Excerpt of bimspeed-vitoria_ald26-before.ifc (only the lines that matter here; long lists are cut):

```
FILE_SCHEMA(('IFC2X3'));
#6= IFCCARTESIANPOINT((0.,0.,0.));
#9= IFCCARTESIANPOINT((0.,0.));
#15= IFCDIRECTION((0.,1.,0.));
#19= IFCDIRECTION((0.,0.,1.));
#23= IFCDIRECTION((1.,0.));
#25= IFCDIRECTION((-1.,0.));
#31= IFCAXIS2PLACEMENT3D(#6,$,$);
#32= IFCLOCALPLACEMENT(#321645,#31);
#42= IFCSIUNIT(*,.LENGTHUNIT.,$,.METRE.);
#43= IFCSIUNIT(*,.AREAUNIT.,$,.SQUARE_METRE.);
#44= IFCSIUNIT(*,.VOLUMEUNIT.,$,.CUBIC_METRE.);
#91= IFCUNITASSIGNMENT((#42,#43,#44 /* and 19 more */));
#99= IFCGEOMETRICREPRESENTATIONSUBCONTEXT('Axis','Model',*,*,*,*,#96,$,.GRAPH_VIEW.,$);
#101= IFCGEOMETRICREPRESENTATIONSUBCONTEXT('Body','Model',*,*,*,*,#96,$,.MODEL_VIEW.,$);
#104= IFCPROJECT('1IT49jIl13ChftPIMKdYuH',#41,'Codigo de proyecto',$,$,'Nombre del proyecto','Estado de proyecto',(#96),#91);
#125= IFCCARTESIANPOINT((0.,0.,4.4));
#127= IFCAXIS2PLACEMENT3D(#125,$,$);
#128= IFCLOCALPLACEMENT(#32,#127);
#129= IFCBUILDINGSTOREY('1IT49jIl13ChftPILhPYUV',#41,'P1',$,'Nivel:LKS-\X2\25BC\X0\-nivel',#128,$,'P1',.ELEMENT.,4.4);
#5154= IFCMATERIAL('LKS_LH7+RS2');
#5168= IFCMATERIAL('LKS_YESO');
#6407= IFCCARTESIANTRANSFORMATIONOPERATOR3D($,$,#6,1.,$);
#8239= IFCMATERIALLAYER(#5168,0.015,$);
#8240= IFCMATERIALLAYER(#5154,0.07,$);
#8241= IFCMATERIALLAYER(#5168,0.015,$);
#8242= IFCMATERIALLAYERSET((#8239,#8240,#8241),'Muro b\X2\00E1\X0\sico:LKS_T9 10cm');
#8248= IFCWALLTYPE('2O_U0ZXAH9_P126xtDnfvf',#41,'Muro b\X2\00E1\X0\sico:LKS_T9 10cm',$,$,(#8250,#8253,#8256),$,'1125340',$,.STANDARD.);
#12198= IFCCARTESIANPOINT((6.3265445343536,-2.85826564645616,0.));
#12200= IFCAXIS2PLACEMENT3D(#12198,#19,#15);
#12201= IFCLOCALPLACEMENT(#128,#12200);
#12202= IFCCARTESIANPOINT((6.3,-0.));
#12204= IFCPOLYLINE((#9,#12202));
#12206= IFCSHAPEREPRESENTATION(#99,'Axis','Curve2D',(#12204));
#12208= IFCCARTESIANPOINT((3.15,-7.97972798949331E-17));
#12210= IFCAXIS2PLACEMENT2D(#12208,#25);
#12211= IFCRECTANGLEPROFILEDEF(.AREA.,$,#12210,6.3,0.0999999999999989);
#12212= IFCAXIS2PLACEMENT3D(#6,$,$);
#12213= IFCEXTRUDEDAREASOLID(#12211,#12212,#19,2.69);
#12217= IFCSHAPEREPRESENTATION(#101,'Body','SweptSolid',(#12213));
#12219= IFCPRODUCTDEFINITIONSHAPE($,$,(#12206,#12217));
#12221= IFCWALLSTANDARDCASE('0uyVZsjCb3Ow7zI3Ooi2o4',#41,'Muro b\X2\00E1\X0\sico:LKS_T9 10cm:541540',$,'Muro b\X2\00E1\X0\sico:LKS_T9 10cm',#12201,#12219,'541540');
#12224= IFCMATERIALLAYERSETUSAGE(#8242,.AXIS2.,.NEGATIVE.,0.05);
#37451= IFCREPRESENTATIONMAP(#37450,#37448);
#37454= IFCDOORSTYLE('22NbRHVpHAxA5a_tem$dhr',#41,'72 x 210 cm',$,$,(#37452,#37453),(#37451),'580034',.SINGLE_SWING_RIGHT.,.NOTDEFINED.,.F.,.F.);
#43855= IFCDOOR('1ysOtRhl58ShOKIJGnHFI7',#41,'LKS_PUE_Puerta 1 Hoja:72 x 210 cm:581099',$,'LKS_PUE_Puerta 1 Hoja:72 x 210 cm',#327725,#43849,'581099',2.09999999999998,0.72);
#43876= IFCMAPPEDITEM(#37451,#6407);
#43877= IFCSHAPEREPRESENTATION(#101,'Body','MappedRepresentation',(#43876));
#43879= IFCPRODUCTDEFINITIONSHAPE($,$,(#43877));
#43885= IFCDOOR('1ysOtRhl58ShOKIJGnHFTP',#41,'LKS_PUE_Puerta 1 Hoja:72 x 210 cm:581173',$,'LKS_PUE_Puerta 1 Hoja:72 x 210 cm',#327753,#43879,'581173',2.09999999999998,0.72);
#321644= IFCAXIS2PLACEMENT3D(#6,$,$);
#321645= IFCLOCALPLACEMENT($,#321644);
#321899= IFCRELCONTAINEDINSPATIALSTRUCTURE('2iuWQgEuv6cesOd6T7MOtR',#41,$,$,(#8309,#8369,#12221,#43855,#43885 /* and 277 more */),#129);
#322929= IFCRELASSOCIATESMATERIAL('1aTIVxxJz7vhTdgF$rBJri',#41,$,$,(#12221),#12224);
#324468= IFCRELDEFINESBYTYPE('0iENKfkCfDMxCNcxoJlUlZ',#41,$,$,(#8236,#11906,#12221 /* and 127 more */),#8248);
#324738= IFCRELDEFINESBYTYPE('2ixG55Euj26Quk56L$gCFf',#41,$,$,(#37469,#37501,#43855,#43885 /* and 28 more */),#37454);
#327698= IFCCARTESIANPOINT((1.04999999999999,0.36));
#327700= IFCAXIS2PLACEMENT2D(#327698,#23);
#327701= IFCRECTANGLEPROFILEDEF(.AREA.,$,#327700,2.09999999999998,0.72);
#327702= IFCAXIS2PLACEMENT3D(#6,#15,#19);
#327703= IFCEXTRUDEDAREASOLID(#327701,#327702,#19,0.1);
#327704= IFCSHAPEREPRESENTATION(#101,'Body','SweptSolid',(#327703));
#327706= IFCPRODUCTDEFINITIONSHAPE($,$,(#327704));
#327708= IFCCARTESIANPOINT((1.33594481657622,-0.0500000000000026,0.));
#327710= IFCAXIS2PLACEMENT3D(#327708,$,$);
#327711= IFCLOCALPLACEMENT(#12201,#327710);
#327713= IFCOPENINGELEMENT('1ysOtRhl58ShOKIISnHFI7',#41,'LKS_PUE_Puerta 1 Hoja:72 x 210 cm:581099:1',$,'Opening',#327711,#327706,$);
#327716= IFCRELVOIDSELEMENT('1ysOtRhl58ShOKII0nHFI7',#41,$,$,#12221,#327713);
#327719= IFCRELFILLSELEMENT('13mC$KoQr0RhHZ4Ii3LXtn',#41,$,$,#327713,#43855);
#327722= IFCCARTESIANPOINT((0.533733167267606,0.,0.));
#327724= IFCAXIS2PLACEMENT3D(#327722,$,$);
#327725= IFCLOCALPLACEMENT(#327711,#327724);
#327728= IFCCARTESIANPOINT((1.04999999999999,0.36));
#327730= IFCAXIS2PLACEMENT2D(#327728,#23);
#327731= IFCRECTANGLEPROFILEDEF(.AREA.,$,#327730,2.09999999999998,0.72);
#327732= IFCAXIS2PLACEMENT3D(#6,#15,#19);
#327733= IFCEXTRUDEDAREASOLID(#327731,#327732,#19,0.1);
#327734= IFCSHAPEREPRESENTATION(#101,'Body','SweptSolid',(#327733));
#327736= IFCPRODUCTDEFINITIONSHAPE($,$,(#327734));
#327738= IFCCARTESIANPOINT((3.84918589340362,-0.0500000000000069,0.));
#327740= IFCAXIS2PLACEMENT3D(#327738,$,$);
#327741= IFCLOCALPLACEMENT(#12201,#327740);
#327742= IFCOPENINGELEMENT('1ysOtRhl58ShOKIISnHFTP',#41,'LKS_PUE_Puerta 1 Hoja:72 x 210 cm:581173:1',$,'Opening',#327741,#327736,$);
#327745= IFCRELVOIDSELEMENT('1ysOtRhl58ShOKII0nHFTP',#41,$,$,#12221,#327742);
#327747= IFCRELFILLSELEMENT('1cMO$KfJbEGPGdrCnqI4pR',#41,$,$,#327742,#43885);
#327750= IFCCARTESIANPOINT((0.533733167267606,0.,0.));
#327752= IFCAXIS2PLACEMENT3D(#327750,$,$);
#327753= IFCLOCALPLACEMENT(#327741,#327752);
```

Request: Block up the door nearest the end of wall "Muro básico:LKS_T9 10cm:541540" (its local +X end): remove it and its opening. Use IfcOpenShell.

```python
import ifcopenshell
import ifcopenshell.api.feature
import ifcopenshell.api.root
import ifcopenshell.geom
import ifcopenshell.util.shape

model = ifcopenshell.open("bimspeed-vitoria_ald26-before.ifc")
settings = ifcopenshell.geom.settings()


def volume(element):
    """Net volume in cubic metres, openings subtracted."""
    shape = ifcopenshell.geom.create_shape(settings, element)
    return ifcopenshell.util.shape.get_volume(shape.geometry)


door = model.by_id(43885)
opening = door.FillsVoids[0].RelatingOpeningElement
wall = opening.VoidsElements[0].RelatingBuildingElement
before = volume(wall)

ifcopenshell.api.root.remove_product(model, product=door)
ifcopenshell.api.feature.remove_feature(model, feature=opening)

after = volume(wall)

print(f"wall volume {before:.3f} -> {after:.3f} m3")

model.write("bimspeed-vitoria_ald26-before_edited.ifc")
```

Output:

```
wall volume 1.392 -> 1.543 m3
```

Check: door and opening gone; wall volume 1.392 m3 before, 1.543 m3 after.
